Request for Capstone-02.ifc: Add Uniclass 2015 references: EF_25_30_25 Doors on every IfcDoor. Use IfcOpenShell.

First a look at what the model holds.

```python
import ifcopenshell

model = ifcopenshell.open("Capstone-02.ifc")
print(model.schema)
print("classifications:", [c.Name for c in model.by_type("IfcClassification")])
for ifc_class in ("IfcDoor", "IfcRoof", "IfcStair", "IfcWall", "IfcWindow"):
    print(ifc_class, len(model.by_type(ifc_class)))
```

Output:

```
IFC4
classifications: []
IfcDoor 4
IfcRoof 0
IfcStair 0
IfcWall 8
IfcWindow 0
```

```python
import ifcopenshell
import ifcopenshell.api.classification

model = ifcopenshell.open("Capstone-02.ifc")

system = ifcopenshell.api.classification.add_classification(model, classification="Uniclass 2015")

codes = {
    "IfcDoor": ("EF_25_30_25", "Doors"),
}
for ifc_class, (code, name) in codes.items():
    products = model.by_type(ifc_class)
    ifcopenshell.api.classification.add_reference(
        model, products=products, classification=system, identification=code, name=name
    )
    print(code, len(products))

model.write("Capstone-02_updated.ifc")
```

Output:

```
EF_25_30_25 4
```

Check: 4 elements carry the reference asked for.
